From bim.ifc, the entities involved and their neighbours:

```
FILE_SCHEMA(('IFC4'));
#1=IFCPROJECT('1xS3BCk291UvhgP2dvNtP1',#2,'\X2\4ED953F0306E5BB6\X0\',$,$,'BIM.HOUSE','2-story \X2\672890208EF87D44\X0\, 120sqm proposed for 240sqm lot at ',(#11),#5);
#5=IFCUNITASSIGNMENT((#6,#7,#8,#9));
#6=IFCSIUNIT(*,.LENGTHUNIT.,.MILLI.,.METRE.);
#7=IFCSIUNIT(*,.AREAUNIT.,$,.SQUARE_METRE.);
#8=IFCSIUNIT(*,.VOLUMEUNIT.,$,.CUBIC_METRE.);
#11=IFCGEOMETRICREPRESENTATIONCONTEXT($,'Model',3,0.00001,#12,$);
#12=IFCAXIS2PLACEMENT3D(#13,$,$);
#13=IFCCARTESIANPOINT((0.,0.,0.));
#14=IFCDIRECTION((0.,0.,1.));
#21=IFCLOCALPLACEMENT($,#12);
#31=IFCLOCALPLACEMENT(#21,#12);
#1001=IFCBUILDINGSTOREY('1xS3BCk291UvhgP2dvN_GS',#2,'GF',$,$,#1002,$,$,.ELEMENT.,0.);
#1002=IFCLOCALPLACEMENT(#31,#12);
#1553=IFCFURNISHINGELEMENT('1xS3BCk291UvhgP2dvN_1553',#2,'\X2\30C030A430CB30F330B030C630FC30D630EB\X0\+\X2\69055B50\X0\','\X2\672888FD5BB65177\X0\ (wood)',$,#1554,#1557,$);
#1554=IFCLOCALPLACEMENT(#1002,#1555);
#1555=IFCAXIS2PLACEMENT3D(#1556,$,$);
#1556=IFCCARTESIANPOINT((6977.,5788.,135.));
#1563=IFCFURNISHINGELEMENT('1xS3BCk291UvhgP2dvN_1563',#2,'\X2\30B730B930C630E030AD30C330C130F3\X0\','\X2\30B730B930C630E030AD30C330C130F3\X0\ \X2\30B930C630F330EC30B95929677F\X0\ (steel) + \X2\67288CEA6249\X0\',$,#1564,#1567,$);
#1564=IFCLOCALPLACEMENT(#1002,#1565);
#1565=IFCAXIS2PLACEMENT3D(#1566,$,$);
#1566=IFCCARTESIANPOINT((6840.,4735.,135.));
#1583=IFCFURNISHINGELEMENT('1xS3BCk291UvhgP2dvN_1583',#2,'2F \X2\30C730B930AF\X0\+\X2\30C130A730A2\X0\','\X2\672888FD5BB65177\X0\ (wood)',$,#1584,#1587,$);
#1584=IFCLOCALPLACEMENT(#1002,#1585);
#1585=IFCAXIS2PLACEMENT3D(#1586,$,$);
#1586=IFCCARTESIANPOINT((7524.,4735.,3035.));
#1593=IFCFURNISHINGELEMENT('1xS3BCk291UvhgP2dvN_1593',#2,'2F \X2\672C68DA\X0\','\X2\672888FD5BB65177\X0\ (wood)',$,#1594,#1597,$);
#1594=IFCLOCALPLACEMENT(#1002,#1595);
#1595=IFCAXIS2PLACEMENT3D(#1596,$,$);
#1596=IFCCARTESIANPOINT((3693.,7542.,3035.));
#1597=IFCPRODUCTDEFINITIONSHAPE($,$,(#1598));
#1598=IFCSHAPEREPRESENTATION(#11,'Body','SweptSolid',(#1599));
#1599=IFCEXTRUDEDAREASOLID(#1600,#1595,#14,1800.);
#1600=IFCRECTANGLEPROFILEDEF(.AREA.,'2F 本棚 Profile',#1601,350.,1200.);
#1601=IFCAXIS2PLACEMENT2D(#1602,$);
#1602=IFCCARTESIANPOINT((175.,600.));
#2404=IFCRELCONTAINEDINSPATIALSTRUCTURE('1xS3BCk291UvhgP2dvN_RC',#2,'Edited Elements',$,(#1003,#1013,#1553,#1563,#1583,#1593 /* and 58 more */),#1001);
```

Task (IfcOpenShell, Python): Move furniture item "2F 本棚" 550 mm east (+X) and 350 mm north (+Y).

```python
import ifcopenshell
import ifcopenshell.api.geometry
import ifcopenshell.util.placement
import ifcopenshell.util.unit

model = ifcopenshell.open("bim.ifc")
unit_scale = ifcopenshell.util.unit.calculate_unit_scale(model)

item = model.by_guid("1xS3BCk291UvhgP2dvN_1593")
matrix = ifcopenshell.util.placement.get_local_placement(item.ObjectPlacement)
matrix[0, 3] += 0.55 / unit_scale
matrix[1, 3] += 0.35 / unit_scale
ifcopenshell.api.geometry.edit_object_placement(model, product=item, matrix=matrix, is_si=False)

print(ifcopenshell.util.placement.get_local_placement(item.ObjectPlacement).round(3) + 0.0)

model.write("bim_rev.ifc")
```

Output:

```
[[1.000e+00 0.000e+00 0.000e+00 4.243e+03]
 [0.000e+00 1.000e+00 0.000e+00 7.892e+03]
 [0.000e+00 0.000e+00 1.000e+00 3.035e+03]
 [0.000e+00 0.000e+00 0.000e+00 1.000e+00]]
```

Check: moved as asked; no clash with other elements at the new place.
